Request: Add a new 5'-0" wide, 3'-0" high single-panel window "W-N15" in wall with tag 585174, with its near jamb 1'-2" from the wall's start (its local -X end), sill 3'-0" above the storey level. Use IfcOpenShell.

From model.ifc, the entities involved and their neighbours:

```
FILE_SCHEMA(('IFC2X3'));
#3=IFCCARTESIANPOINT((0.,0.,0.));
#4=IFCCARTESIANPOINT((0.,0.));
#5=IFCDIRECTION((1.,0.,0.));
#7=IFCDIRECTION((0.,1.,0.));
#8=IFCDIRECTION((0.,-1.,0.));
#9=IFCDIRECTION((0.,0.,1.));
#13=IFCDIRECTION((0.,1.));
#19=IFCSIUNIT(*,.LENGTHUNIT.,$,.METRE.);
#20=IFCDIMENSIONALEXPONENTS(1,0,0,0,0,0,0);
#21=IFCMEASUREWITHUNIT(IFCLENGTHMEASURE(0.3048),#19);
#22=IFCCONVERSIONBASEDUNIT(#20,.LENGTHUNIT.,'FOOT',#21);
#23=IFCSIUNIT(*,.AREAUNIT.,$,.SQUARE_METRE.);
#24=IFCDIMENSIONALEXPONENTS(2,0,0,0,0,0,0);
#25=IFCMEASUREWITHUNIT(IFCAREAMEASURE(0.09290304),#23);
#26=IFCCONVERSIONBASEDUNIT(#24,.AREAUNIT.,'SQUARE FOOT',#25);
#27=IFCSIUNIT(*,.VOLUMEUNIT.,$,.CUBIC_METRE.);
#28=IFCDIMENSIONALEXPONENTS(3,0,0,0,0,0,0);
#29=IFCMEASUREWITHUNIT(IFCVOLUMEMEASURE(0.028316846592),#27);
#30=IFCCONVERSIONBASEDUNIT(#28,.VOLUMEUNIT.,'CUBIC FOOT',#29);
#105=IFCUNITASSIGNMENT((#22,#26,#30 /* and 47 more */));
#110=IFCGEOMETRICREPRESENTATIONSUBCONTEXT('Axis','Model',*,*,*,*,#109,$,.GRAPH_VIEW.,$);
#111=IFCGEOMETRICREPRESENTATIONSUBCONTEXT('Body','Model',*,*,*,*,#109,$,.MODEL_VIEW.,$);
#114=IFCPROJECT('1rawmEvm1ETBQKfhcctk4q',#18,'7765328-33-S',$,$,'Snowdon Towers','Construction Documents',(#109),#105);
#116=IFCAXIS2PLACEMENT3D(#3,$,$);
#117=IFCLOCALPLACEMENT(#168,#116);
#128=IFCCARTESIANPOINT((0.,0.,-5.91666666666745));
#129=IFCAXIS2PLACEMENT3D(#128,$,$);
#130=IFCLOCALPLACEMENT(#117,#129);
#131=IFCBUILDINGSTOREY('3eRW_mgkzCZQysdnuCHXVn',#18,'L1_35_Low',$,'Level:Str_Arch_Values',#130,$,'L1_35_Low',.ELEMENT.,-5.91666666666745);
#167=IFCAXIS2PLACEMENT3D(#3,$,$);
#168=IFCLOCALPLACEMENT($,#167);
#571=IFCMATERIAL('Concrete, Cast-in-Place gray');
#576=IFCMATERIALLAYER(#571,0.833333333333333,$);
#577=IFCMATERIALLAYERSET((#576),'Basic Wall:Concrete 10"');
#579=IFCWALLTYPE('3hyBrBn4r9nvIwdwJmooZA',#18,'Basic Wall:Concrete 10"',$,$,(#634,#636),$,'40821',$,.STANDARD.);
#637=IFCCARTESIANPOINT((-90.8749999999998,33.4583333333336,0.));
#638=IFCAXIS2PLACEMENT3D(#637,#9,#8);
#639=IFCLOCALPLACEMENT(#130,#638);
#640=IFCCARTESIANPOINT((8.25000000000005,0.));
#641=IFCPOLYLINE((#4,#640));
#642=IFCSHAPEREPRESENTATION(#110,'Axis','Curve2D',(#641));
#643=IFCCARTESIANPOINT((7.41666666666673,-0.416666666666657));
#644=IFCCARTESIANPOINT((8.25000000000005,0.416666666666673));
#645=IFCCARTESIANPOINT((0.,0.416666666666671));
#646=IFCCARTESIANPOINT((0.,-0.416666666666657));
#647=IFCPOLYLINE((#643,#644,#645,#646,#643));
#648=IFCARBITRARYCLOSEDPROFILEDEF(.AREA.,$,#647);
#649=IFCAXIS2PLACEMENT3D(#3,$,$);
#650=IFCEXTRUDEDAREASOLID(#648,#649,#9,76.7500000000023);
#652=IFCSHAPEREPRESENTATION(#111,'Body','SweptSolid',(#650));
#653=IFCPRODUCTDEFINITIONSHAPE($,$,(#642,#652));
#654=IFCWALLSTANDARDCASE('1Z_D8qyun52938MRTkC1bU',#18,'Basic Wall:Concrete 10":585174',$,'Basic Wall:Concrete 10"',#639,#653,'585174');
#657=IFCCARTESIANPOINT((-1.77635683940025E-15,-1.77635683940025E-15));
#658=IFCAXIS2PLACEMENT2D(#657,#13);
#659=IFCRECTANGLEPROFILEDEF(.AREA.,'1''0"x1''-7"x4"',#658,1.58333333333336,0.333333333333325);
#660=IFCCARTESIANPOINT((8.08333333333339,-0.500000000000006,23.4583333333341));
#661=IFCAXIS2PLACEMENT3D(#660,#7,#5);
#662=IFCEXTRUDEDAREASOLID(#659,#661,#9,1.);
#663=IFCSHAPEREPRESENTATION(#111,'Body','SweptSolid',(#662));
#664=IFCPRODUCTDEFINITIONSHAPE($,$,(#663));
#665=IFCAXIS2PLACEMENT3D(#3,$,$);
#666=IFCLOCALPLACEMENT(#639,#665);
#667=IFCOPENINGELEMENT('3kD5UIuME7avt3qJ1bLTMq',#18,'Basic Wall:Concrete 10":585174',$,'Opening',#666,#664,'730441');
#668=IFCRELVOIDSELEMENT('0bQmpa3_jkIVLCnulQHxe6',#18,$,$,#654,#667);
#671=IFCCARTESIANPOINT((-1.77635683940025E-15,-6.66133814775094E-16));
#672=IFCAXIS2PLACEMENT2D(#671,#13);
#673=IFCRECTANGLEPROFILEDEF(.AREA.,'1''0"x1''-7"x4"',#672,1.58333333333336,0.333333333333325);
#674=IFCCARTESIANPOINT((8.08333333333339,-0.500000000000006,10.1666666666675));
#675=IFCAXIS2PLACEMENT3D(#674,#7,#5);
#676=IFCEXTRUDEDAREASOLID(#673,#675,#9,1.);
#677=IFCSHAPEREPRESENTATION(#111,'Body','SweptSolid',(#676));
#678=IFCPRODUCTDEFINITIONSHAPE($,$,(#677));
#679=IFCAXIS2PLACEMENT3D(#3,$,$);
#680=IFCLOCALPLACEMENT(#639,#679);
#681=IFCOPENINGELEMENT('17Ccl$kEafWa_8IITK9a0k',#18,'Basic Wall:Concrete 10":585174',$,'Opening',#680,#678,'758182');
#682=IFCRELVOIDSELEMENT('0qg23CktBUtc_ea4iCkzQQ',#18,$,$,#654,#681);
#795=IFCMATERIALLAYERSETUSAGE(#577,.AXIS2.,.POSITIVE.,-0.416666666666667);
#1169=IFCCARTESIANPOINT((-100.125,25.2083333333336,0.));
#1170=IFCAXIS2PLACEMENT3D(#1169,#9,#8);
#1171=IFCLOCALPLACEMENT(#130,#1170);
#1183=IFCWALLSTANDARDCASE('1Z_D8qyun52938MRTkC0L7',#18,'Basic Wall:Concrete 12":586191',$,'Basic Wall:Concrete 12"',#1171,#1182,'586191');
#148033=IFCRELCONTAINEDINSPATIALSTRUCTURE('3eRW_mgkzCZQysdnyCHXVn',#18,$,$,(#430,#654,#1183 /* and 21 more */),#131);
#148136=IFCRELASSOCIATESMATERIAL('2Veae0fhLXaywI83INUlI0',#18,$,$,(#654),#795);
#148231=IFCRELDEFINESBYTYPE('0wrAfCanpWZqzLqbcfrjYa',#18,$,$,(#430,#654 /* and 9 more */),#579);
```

```python
import numpy as np
import ifcopenshell
import ifcopenshell.api.feature
import ifcopenshell.api.geometry
import ifcopenshell.api.root
import ifcopenshell.api.spatial
import ifcopenshell.api.type
import ifcopenshell.geom
import ifcopenshell.util.element
import ifcopenshell.util.placement
import ifcopenshell.util.representation
import ifcopenshell.util.shape
import ifcopenshell.util.unit

model = ifcopenshell.open("model.ifc")
unit_scale = ifcopenshell.util.unit.calculate_unit_scale(model)
settings = ifcopenshell.geom.settings()


def volume(element):
    """Net volume in cubic metres, openings subtracted."""
    shape = ifcopenshell.geom.create_shape(settings, element)
    return ifcopenshell.util.shape.get_volume(shape.geometry)


wall = model.by_guid("1Z_D8qyun52938MRTkC1bU")
storey = ifcopenshell.util.element.get_container(wall, ifc_class="IfcBuildingStorey")
context = ifcopenshell.util.representation.get_context(model, "Model", "Body", "MODEL_VIEW")
before = volume(wall)

width, height, from_end, sill = 1.524, 0.9144, 0.3556, 0.9144  # metres

# The wall runs along its own X axis, and the end named is its -X end.
wall_shape = ifcopenshell.geom.create_shape(settings, wall)
x, y, z = ifcopenshell.util.shape.get_vertices(wall_shape.geometry).T
start = x.min() + from_end
face, thickness = float(y.min()), float(y.max() - y.min())
wall_matrix = ifcopenshell.util.placement.get_local_placement(wall.ObjectPlacement)
level = ifcopenshell.util.placement.get_local_placement(storey.ObjectPlacement)[2, 3]


def in_wall(x, y):
    """Placement at x, y metres in the wall's axes, at sill height."""
    matrix = wall_matrix.copy()
    matrix[:, 3] = wall_matrix @ np.array([x / unit_scale, y / unit_scale, 0.0, 1.0])
    matrix[2, 3] = level + sill / unit_scale
    return matrix


# Opening: a box that overshoots both wall faces by 50 mm.
opening = ifcopenshell.api.root.create_entity(model, ifc_class="IfcOpeningElement")
box = ifcopenshell.api.geometry.add_wall_representation(
    model, context=context, length=width, height=height, thickness=thickness + 0.1
)
ifcopenshell.api.geometry.assign_representation(model, product=opening, representation=box)
ifcopenshell.api.geometry.edit_object_placement(model, product=opening, matrix=in_wall(start, face - 0.05), is_si=False)
ifcopenshell.api.feature.add_feature(model, feature=opening, element=wall)

window = ifcopenshell.api.root.create_entity(model, ifc_class="IfcWindow", name="W-N15")
window.OverallWidth, window.OverallHeight = width / unit_scale, height / unit_scale
body = ifcopenshell.api.geometry.add_window_representation(
    model,
    context=context,
    overall_width=window.OverallWidth,
    overall_height=window.OverallHeight,
    partition_type="SINGLE_PANEL",
)
ifcopenshell.api.geometry.assign_representation(model, product=window, representation=body)
ifcopenshell.api.spatial.assign_container(model, products=[window], relating_structure=storey)
fills = ifcopenshell.api.feature.add_filling(model, opening=opening, element=window)
fills.OwnerHistory = window.OwnerHistory  # required in IFC2X3

# IFC2X3 keeps the operation on the window style.
style = ifcopenshell.api.root.create_entity(model, ifc_class="IfcWindowStyle", name="W-N15")
style.OperationType, style.ConstructionType = "SINGLE_PANEL", "NOTDEFINED"
style.ParameterTakesPrecedence = style.Sizeable = False
ifcopenshell.api.type.assign_type(model, related_objects=[window], relating_type=style)

# Centre the window in the wall's thickness.
ifcopenshell.api.geometry.edit_object_placement(model, product=window, matrix=in_wall(start, face), is_si=False)
window_shape = ifcopenshell.geom.create_shape(settings, window)
depth = ifcopenshell.util.shape.get_vertices(window_shape.geometry)[:, 1]
offset = face + thickness / 2 - (depth.min() + depth.max()) / 2
ifcopenshell.api.geometry.edit_object_placement(model, product=window, matrix=in_wall(start, offset), is_si=False)

after = volume(wall)

print(f"wall volume {before:.3f} -> {after:.3f} m3")

model.write("model_updated.ifc")
```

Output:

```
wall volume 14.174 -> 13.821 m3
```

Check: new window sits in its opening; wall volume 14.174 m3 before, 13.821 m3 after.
